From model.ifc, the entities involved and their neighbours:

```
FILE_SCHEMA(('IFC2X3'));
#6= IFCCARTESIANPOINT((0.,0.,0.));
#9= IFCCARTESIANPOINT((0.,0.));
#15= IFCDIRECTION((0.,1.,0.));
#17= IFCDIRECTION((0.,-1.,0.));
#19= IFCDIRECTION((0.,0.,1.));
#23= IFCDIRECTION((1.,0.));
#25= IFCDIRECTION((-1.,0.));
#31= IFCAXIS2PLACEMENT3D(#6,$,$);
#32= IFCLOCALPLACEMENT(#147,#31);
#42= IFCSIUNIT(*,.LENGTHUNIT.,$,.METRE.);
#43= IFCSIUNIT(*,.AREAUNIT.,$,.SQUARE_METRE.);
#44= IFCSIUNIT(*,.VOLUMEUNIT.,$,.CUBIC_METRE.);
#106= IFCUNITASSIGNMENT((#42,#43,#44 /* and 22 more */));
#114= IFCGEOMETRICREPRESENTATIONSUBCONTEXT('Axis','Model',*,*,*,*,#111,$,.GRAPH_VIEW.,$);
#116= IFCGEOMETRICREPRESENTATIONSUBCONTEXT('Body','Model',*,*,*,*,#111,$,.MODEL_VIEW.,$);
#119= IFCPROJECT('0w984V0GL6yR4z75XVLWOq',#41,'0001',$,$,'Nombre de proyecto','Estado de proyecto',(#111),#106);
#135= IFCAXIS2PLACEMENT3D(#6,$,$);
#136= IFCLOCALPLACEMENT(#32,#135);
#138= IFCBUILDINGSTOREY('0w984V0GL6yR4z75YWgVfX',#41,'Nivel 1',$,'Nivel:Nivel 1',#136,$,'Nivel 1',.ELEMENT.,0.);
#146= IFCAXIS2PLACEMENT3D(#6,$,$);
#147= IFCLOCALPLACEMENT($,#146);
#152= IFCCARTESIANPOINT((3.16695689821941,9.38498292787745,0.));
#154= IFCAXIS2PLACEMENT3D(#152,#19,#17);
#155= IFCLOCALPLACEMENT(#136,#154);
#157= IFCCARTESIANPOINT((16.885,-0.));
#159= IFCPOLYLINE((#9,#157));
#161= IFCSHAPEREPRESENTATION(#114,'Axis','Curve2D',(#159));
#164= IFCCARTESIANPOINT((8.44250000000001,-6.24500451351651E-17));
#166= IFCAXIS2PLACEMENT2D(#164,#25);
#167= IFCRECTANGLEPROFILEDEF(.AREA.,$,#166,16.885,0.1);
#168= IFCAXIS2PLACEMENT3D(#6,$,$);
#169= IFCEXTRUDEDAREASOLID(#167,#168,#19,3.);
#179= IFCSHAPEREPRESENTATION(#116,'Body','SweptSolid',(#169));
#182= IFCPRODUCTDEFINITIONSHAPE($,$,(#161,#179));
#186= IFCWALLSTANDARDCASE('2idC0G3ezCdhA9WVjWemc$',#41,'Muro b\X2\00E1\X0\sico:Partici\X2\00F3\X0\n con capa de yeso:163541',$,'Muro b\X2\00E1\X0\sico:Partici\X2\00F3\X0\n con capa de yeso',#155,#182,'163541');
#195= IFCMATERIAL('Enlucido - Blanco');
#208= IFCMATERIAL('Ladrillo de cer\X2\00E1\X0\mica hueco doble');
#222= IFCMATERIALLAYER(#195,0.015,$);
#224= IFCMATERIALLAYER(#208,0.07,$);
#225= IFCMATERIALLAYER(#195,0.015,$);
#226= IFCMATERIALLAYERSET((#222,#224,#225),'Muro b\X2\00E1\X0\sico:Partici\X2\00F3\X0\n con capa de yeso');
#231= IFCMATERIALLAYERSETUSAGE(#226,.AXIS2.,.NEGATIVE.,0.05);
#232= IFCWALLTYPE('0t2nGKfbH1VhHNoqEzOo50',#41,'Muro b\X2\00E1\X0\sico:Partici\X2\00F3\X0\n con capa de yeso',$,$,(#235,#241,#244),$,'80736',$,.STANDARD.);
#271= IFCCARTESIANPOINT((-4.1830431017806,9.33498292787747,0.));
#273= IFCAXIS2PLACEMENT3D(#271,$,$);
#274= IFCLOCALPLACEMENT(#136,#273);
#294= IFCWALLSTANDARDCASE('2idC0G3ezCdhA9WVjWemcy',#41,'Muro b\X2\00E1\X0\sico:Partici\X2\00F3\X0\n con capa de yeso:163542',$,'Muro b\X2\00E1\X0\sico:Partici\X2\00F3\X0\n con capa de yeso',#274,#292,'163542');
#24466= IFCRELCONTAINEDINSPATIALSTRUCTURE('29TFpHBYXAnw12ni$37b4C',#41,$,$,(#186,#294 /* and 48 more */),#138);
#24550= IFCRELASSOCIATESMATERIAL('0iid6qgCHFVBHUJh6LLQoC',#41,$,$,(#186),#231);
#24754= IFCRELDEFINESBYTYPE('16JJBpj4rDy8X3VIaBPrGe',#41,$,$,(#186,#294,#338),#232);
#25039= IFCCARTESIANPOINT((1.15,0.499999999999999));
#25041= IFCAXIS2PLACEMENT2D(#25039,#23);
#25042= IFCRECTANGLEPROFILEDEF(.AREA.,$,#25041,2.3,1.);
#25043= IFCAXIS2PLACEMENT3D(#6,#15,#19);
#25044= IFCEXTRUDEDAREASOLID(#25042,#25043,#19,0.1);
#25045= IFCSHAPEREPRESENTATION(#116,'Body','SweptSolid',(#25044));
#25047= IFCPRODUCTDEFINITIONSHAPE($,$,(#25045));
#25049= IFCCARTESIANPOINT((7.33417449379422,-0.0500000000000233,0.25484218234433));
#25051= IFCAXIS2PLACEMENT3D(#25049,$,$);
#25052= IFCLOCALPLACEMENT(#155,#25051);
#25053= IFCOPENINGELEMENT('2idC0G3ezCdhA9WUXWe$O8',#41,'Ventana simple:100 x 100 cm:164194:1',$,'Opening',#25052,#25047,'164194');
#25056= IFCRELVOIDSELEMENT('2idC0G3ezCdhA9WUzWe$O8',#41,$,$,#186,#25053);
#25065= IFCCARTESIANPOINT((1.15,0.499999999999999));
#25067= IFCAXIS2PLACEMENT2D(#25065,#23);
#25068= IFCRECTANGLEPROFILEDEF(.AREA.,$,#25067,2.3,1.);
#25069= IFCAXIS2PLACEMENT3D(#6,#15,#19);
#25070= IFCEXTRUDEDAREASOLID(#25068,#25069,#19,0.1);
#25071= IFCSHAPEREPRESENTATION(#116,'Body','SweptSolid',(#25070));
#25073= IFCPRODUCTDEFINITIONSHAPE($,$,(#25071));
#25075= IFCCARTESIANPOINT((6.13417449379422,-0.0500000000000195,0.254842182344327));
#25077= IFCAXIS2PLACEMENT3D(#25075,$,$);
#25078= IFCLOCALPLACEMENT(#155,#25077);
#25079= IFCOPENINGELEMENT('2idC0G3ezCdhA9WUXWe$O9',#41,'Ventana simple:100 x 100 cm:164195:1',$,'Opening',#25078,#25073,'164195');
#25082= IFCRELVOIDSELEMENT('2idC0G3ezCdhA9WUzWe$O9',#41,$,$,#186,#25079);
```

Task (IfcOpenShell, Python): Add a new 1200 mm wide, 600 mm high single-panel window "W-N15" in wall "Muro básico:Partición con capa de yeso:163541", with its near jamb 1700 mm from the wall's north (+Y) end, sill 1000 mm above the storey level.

```python
import numpy as np
import ifcopenshell
import ifcopenshell.api.feature
import ifcopenshell.api.geometry
import ifcopenshell.api.root
import ifcopenshell.api.spatial
import ifcopenshell.api.type
import ifcopenshell.geom
import ifcopenshell.util.element
import ifcopenshell.util.placement
import ifcopenshell.util.representation
import ifcopenshell.util.shape
import ifcopenshell.util.unit

model = ifcopenshell.open("model.ifc")
unit_scale = ifcopenshell.util.unit.calculate_unit_scale(model)
settings = ifcopenshell.geom.settings()


def volume(element):
    """Net volume in cubic metres, openings subtracted."""
    shape = ifcopenshell.geom.create_shape(settings, element)
    return ifcopenshell.util.shape.get_volume(shape.geometry)


wall = model.by_guid("2idC0G3ezCdhA9WVjWemc$")
storey = ifcopenshell.util.element.get_container(wall, ifc_class="IfcBuildingStorey")
context = ifcopenshell.util.representation.get_context(model, "Model", "Body", "MODEL_VIEW")
before = volume(wall)

width, height, from_end, sill = 1.2, 0.6, 1.7, 1  # metres

# The wall runs along its own X axis, and the end named is its -X end.
wall_shape = ifcopenshell.geom.create_shape(settings, wall)
x, y, z = ifcopenshell.util.shape.get_vertices(wall_shape.geometry).T
start = x.min() + from_end
face, thickness = float(y.min()), float(y.max() - y.min())
wall_matrix = ifcopenshell.util.placement.get_local_placement(wall.ObjectPlacement)
level = ifcopenshell.util.placement.get_local_placement(storey.ObjectPlacement)[2, 3]


def in_wall(x, y):
    """Placement at x, y metres in the wall's axes, at sill height."""
    matrix = wall_matrix.copy()
    matrix[:, 3] = wall_matrix @ np.array([x / unit_scale, y / unit_scale, 0.0, 1.0])
    matrix[2, 3] = level + sill / unit_scale
    return matrix


# Opening: a box that overshoots both wall faces by 50 mm.
opening = ifcopenshell.api.root.create_entity(model, ifc_class="IfcOpeningElement")
box = ifcopenshell.api.geometry.add_wall_representation(
    model, context=context, length=width, height=height, thickness=thickness + 0.1
)
ifcopenshell.api.geometry.assign_representation(model, product=opening, representation=box)
ifcopenshell.api.geometry.edit_object_placement(model, product=opening, matrix=in_wall(start, face - 0.05), is_si=False)
ifcopenshell.api.feature.add_feature(model, feature=opening, element=wall)

window = ifcopenshell.api.root.create_entity(model, ifc_class="IfcWindow", name="W-N15")
window.OverallWidth, window.OverallHeight = width / unit_scale, height / unit_scale
body = ifcopenshell.api.geometry.add_window_representation(
    model,
    context=context,
    overall_width=window.OverallWidth,
    overall_height=window.OverallHeight,
    partition_type="SINGLE_PANEL",
)
ifcopenshell.api.geometry.assign_representation(model, product=window, representation=body)
ifcopenshell.api.spatial.assign_container(model, products=[window], relating_structure=storey)
fills = ifcopenshell.api.feature.add_filling(model, opening=opening, element=window)
fills.OwnerHistory = window.OwnerHistory  # required in IFC2X3

# IFC2X3 keeps the operation on the window style.
style = ifcopenshell.api.root.create_entity(model, ifc_class="IfcWindowStyle", name="W-N15")
style.OperationType, style.ConstructionType = "SINGLE_PANEL", "NOTDEFINED"
style.ParameterTakesPrecedence = style.Sizeable = False
ifcopenshell.api.type.assign_type(model, related_objects=[window], relating_type=style)

# Centre the window in the wall's thickness.
ifcopenshell.api.geometry.edit_object_placement(model, product=window, matrix=in_wall(start, face), is_si=False)
window_shape = ifcopenshell.geom.create_shape(settings, window)
depth = ifcopenshell.util.shape.get_vertices(window_shape.geometry)[:, 1]
offset = face + thickness / 2 - (depth.min() + depth.max()) / 2
ifcopenshell.api.geometry.edit_object_placement(model, product=window, matrix=in_wall(start, offset), is_si=False)

after = volume(wall)

print(f"wall volume {before:.3f} -> {after:.3f} m3")

model.write("model_updated.ifc")
```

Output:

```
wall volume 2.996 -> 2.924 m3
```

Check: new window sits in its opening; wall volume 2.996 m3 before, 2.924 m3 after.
